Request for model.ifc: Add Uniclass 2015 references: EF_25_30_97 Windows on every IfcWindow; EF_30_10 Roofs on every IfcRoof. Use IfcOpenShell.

First a look at what the model holds.

```python
import ifcopenshell

model = ifcopenshell.open("model.ifc")
print(model.schema)
print("classifications:", [c.Name for c in model.by_type("IfcClassification")])
for ifc_class in ("IfcDoor", "IfcRoof", "IfcStair", "IfcWall", "IfcWindow"):
    print(ifc_class, len(model.by_type(ifc_class)))
```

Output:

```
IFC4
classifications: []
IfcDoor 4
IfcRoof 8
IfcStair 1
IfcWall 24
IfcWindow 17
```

```python
import ifcopenshell
import ifcopenshell.api.classification

model = ifcopenshell.open("model.ifc")

system = ifcopenshell.api.classification.add_classification(model, classification="Uniclass 2015")

codes = {
    "IfcWindow": ("EF_25_30_97", "Windows"),
    "IfcRoof": ("EF_30_10", "Roofs"),
}
for ifc_class, (code, name) in codes.items():
    products = model.by_type(ifc_class)
    ifcopenshell.api.classification.add_reference(
        model, products=products, classification=system, identification=code, name=name
    )
    print(code, len(products))

model.write("model_v2.ifc")
```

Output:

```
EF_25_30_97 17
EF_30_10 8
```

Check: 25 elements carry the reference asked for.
